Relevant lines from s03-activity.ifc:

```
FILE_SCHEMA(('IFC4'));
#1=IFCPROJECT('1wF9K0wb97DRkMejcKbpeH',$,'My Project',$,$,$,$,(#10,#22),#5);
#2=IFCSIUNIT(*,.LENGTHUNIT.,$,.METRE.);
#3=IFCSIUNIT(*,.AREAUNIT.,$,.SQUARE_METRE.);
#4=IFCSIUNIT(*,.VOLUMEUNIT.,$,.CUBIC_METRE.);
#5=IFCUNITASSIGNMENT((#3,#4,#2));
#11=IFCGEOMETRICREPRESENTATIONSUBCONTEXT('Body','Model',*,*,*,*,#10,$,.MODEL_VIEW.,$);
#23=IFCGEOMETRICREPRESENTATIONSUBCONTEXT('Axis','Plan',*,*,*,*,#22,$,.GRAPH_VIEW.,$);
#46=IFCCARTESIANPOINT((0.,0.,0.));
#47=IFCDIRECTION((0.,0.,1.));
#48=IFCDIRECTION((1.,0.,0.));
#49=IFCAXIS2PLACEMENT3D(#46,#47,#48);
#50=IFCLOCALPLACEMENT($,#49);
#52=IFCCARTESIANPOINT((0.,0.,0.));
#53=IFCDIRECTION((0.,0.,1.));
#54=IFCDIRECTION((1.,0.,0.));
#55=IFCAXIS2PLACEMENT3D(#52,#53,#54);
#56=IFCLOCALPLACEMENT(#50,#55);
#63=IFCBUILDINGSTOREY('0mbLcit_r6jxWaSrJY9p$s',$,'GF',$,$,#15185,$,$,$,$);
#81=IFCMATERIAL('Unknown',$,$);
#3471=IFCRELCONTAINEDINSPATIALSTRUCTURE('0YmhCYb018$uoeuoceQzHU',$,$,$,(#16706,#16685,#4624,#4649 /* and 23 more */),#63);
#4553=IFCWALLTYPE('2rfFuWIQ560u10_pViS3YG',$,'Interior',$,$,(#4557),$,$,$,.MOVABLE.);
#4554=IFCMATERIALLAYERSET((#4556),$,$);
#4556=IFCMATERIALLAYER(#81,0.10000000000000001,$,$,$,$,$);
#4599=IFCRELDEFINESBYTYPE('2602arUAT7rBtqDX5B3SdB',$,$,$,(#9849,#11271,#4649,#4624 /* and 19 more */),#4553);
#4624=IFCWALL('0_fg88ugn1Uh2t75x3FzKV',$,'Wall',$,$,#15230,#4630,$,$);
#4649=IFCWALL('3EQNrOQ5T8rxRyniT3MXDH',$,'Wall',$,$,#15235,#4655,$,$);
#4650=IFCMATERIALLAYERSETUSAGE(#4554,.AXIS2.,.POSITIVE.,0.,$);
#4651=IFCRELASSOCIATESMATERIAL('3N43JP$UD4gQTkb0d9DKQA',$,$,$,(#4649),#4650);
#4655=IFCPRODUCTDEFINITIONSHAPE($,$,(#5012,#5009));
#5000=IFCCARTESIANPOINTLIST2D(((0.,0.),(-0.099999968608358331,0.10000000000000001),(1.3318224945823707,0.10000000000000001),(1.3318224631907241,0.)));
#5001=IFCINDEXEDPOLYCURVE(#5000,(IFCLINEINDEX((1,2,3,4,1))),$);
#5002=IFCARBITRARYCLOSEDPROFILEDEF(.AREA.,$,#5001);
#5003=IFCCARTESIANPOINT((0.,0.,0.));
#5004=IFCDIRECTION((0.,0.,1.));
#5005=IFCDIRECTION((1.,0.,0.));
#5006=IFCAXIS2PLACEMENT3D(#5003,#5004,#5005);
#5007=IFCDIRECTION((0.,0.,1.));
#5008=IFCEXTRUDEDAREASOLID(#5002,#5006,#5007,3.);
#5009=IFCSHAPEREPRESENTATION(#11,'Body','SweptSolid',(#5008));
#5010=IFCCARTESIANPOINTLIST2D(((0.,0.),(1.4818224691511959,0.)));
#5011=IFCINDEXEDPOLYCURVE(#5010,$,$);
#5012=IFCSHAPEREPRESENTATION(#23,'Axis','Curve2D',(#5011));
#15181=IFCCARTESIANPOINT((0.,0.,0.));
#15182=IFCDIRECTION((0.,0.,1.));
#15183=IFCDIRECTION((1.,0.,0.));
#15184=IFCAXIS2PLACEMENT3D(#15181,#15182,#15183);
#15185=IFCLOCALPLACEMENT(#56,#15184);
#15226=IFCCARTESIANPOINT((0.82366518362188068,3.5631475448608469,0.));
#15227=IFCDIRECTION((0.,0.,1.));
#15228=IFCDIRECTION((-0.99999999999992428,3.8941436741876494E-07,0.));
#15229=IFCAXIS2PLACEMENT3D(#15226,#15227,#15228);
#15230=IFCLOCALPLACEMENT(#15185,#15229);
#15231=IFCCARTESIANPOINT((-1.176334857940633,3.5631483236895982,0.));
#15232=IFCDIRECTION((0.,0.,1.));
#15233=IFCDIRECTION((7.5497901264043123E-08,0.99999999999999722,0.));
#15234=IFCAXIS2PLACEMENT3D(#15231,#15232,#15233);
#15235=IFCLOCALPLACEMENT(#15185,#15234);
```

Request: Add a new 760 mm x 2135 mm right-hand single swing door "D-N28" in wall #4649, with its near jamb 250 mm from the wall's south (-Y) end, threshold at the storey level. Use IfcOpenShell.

```python
import numpy as np
import ifcopenshell
import ifcopenshell.api.feature
import ifcopenshell.api.geometry
import ifcopenshell.api.root
import ifcopenshell.api.spatial
import ifcopenshell.geom
import ifcopenshell.util.element
import ifcopenshell.util.placement
import ifcopenshell.util.representation
import ifcopenshell.util.shape
import ifcopenshell.util.unit

model = ifcopenshell.open("s03-activity.ifc")
unit_scale = ifcopenshell.util.unit.calculate_unit_scale(model)
settings = ifcopenshell.geom.settings()


def volume(element):
    """Net volume in cubic metres, openings subtracted."""
    shape = ifcopenshell.geom.create_shape(settings, element)
    return ifcopenshell.util.shape.get_volume(shape.geometry)


wall = model.by_guid("3EQNrOQ5T8rxRyniT3MXDH")
storey = ifcopenshell.util.element.get_container(wall, ifc_class="IfcBuildingStorey")
context = ifcopenshell.util.representation.get_context(model, "Model", "Body", "MODEL_VIEW")
before = volume(wall)

width, height, from_end, sill = 0.76, 2.135, 0.25, 0.0  # metres

# The wall runs along its own X axis, and the end named is its -X end.
wall_shape = ifcopenshell.geom.create_shape(settings, wall)
x, y, z = ifcopenshell.util.shape.get_vertices(wall_shape.geometry).T
start = x.min() + from_end
face, thickness = float(y.min()), float(y.max() - y.min())
wall_matrix = ifcopenshell.util.placement.get_local_placement(wall.ObjectPlacement)
level = ifcopenshell.util.placement.get_local_placement(storey.ObjectPlacement)[2, 3]


def in_wall(x, y):
    """Placement at x, y metres in the wall's axes, at sill height."""
    matrix = wall_matrix.copy()
    matrix[:, 3] = wall_matrix @ np.array([x / unit_scale, y / unit_scale, 0.0, 1.0])
    matrix[2, 3] = level + sill / unit_scale
    return matrix


# Opening: a box that overshoots both wall faces by 50 mm.
opening = ifcopenshell.api.root.create_entity(model, ifc_class="IfcOpeningElement", predefined_type="OPENING")
box = ifcopenshell.api.geometry.add_wall_representation(
    model, context=context, length=width, height=height, thickness=thickness + 0.1
)
ifcopenshell.api.geometry.assign_representation(model, product=opening, representation=box)
ifcopenshell.api.geometry.edit_object_placement(model, product=opening, matrix=in_wall(start, face - 0.05), is_si=False)
ifcopenshell.api.feature.add_feature(model, feature=opening, element=wall)

door = ifcopenshell.api.root.create_entity(model, ifc_class="IfcDoor", name="D-N28", predefined_type="DOOR")
door.OverallWidth, door.OverallHeight = width / unit_scale, height / unit_scale
door.OperationType = "SINGLE_SWING_RIGHT"
body = ifcopenshell.api.geometry.add_door_representation(
    model,
    context=context,
    overall_width=door.OverallWidth,
    overall_height=door.OverallHeight,
    operation_type="SINGLE_SWING_RIGHT",
    lining_properties={"LiningDepth": thickness / unit_scale, "ThresholdDepth": thickness / unit_scale},
)
ifcopenshell.api.geometry.assign_representation(model, product=door, representation=body)
ifcopenshell.api.spatial.assign_container(model, products=[door], relating_structure=storey)
ifcopenshell.api.feature.add_filling(model, opening=opening, element=door)

# The lining spans the wall, so the door starts at the wall face.
ifcopenshell.api.geometry.edit_object_placement(model, product=door, matrix=in_wall(start, face), is_si=False)

after = volume(wall)

print(f"wall volume {before:.3f} -> {after:.3f} m3")

model.write("s03-activity_updated.ifc")
```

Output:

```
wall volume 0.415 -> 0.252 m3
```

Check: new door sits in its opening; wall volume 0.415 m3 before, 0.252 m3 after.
